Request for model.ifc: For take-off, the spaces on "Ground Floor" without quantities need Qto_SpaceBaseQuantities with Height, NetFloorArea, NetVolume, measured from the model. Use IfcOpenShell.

First a look at what the model holds.

```python
import ifcopenshell
import ifcopenshell.util.element
import ifcopenshell.util.unit

model = ifcopenshell.open("model.ifc")
print(model.schema)
for unit_type in ("LENGTHUNIT", "AREAUNIT", "VOLUMEUNIT"):
    print(unit_type, ifcopenshell.util.unit.calculate_unit_scale(model, unit_type))
storey = next(s for s in model.by_type("IfcBuildingStorey") if s.Name == "Ground Floor")
spaces = [e for e in ifcopenshell.util.element.get_decomposition(storey) if e.is_a("IfcSpace")]
for e in sorted(spaces, key=lambda e: e.id()):
    print(e.id(), e.is_a(), e.Name, list(ifcopenshell.util.element.get_psets(e, qtos_only=True)), sep=" | ")
```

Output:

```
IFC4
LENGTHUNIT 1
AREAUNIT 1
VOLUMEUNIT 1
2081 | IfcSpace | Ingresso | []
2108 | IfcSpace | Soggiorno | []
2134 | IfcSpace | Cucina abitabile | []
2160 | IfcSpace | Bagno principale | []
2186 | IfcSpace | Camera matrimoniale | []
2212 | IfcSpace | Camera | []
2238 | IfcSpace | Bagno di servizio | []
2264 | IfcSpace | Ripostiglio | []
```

```python
import ifcopenshell
import ifcopenshell.api.pset
import ifcopenshell.geom
import ifcopenshell.util.element
import ifcopenshell.util.shape
import ifcopenshell.util.unit

model = ifcopenshell.open("model.ifc")
unit_scale = ifcopenshell.util.unit.calculate_unit_scale(model)
area_scale = ifcopenshell.util.unit.calculate_unit_scale(model, "AREAUNIT")
volume_scale = ifcopenshell.util.unit.calculate_unit_scale(model, "VOLUMEUNIT")
settings = ifcopenshell.geom.settings()

storey = next(s for s in model.by_type("IfcBuildingStorey") if s.Name == "Ground Floor")
spaces = [e for e in ifcopenshell.util.element.get_decomposition(storey) if e.is_a("IfcSpace")]

for e in sorted(spaces, key=lambda e: e.id()):
    if ifcopenshell.util.element.get_psets(e, qtos_only=True, should_inherit=False):
        continue
    # Geometry comes back in metres, in the element's own axes.
    shape = ifcopenshell.geom.create_shape(settings, e)
    values = {
        "Height": ifcopenshell.util.shape.get_z(shape.geometry) / unit_scale,
        "NetFloorArea": ifcopenshell.util.shape.get_footprint_area(shape.geometry) / area_scale,
        "NetVolume": ifcopenshell.util.shape.get_volume(shape.geometry) / volume_scale,
    }
    qto = ifcopenshell.api.pset.add_qto(model, product=e, name="Qto_SpaceBaseQuantities")
    ifcopenshell.api.pset.edit_qto(model, qto=qto, properties=values)
    print(e.id(), {k: round(v, 3) for k, v in values.items()})

model.write("model-out.ifc")
```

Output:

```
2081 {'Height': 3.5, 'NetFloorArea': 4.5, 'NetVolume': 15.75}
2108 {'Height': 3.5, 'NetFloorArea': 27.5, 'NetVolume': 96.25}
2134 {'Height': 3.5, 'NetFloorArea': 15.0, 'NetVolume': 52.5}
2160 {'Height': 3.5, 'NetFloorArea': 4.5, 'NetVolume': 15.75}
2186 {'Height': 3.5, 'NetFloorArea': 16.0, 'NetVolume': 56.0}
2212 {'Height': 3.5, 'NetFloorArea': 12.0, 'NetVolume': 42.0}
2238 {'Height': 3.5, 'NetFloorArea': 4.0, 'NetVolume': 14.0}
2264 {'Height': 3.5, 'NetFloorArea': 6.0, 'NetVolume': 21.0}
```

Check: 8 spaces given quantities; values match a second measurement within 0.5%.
